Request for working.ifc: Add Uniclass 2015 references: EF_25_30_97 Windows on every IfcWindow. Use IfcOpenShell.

First a look at what the model holds.

```python
import ifcopenshell

model = ifcopenshell.open("working.ifc")
print(model.schema)
print("classifications:", [c.Name for c in model.by_type("IfcClassification")])
for ifc_class in ("IfcDoor", "IfcRoof", "IfcStair", "IfcWall", "IfcWindow"):
    print(ifc_class, len(model.by_type(ifc_class)))
```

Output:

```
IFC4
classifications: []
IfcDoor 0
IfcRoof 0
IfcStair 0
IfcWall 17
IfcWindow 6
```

```python
import ifcopenshell
import ifcopenshell.api.classification

model = ifcopenshell.open("working.ifc")

system = ifcopenshell.api.classification.add_classification(model, classification="Uniclass 2015")

codes = {
    "IfcWindow": ("EF_25_30_97", "Windows"),
}
for ifc_class, (code, name) in codes.items():
    products = model.by_type(ifc_class)
    ifcopenshell.api.classification.add_reference(
        model, products=products, classification=system, identification=code, name=name
    )
    print(code, len(products))

model.write("working_rev.ifc")
```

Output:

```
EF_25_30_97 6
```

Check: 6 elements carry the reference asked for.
